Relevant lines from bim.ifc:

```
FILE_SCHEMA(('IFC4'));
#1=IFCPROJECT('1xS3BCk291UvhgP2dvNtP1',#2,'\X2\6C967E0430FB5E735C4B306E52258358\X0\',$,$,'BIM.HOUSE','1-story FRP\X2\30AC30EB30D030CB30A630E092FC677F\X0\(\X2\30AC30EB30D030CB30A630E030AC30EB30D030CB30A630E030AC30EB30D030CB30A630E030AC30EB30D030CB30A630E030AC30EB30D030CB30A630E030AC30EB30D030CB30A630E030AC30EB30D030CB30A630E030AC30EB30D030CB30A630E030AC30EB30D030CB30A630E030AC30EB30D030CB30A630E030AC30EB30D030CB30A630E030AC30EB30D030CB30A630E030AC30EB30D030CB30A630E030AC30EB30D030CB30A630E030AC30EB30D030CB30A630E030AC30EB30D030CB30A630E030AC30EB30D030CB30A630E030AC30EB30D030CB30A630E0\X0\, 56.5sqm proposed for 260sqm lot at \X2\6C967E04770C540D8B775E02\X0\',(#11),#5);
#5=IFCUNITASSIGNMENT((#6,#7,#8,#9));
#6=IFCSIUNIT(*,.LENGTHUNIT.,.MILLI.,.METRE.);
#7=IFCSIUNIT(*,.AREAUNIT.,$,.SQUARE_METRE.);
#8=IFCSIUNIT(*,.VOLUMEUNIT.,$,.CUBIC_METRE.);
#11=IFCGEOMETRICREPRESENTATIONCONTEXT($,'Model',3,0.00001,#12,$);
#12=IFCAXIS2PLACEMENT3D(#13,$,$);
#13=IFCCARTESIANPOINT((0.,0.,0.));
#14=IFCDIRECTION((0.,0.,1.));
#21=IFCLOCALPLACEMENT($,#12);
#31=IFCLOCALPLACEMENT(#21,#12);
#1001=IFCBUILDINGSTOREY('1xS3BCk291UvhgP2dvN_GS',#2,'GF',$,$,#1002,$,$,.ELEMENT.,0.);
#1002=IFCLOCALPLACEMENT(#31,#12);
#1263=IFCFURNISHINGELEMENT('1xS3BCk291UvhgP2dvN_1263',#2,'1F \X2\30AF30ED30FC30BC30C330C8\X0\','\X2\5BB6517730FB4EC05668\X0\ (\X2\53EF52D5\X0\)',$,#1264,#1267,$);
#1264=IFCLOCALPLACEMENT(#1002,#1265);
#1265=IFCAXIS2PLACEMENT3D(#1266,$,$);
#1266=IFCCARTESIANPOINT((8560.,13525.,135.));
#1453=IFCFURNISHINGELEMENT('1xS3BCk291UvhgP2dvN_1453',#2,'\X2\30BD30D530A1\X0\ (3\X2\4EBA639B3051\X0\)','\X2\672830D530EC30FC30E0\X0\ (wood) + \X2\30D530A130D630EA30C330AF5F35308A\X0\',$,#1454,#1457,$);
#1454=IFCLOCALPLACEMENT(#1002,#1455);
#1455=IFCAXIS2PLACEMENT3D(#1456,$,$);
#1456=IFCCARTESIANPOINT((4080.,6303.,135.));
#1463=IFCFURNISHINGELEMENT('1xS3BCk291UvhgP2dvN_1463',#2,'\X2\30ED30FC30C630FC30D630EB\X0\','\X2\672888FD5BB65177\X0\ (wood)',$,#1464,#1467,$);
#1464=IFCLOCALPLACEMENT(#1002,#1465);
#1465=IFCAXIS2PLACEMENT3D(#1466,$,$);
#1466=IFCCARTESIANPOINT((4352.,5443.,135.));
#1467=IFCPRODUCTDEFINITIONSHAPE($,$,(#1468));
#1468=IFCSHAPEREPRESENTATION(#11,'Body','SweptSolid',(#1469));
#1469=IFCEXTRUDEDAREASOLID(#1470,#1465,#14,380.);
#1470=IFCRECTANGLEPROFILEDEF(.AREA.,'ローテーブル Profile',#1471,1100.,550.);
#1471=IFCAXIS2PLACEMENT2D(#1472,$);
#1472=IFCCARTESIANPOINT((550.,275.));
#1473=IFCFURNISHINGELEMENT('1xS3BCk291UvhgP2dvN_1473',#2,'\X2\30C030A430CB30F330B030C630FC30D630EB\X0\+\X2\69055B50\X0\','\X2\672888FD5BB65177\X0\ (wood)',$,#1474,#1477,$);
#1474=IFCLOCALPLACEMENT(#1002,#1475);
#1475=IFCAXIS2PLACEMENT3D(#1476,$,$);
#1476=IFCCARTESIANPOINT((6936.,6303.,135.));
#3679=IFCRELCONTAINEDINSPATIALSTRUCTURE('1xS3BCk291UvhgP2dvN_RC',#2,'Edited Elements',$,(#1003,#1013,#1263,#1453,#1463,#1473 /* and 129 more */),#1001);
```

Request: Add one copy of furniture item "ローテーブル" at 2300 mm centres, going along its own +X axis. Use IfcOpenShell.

```python
import ifcopenshell
import ifcopenshell.api.geometry
import ifcopenshell.api.root
import ifcopenshell.util.element
import ifcopenshell.util.placement

model = ifcopenshell.open("bim.ifc")


def reuse_history(source, copy):
    """copy_class also copies each property set's owner history, people and application; keep the originals."""
    for rel in copy.IsDefinedBy:
        if rel.is_a("IfcRelDefinesByProperties") and (history := rel.RelatingPropertyDefinition.OwnerHistory):
            rel.RelatingPropertyDefinition.OwnerHistory = source.OwnerHistory
            ifcopenshell.util.element.remove_deep2(model, history)


source = model.by_guid("1xS3BCk291UvhgP2dvN_1463")
base = ifcopenshell.util.placement.get_local_placement(source.ObjectPlacement)
step = base[:3, 0] * 2300.0

for i in range(1, 2):
    copy = ifcopenshell.api.root.copy_class(model, product=source)
    copy.Representation = ifcopenshell.util.element.copy_deep(
        model, source.Representation, exclude=["IfcGeometricRepresentationContext", "IfcRepresentationMap"]
    )
    reuse_history(source, copy)
    matrix = base.copy()
    matrix[:3, 3] += i * step
    print("added at", matrix[:3, 3].round(3) + 0.0)
    ifcopenshell.api.geometry.edit_object_placement(model, product=copy, matrix=matrix, is_si=False)

model.write("bim-out.ifc")
```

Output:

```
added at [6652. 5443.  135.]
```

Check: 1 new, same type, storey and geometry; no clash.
